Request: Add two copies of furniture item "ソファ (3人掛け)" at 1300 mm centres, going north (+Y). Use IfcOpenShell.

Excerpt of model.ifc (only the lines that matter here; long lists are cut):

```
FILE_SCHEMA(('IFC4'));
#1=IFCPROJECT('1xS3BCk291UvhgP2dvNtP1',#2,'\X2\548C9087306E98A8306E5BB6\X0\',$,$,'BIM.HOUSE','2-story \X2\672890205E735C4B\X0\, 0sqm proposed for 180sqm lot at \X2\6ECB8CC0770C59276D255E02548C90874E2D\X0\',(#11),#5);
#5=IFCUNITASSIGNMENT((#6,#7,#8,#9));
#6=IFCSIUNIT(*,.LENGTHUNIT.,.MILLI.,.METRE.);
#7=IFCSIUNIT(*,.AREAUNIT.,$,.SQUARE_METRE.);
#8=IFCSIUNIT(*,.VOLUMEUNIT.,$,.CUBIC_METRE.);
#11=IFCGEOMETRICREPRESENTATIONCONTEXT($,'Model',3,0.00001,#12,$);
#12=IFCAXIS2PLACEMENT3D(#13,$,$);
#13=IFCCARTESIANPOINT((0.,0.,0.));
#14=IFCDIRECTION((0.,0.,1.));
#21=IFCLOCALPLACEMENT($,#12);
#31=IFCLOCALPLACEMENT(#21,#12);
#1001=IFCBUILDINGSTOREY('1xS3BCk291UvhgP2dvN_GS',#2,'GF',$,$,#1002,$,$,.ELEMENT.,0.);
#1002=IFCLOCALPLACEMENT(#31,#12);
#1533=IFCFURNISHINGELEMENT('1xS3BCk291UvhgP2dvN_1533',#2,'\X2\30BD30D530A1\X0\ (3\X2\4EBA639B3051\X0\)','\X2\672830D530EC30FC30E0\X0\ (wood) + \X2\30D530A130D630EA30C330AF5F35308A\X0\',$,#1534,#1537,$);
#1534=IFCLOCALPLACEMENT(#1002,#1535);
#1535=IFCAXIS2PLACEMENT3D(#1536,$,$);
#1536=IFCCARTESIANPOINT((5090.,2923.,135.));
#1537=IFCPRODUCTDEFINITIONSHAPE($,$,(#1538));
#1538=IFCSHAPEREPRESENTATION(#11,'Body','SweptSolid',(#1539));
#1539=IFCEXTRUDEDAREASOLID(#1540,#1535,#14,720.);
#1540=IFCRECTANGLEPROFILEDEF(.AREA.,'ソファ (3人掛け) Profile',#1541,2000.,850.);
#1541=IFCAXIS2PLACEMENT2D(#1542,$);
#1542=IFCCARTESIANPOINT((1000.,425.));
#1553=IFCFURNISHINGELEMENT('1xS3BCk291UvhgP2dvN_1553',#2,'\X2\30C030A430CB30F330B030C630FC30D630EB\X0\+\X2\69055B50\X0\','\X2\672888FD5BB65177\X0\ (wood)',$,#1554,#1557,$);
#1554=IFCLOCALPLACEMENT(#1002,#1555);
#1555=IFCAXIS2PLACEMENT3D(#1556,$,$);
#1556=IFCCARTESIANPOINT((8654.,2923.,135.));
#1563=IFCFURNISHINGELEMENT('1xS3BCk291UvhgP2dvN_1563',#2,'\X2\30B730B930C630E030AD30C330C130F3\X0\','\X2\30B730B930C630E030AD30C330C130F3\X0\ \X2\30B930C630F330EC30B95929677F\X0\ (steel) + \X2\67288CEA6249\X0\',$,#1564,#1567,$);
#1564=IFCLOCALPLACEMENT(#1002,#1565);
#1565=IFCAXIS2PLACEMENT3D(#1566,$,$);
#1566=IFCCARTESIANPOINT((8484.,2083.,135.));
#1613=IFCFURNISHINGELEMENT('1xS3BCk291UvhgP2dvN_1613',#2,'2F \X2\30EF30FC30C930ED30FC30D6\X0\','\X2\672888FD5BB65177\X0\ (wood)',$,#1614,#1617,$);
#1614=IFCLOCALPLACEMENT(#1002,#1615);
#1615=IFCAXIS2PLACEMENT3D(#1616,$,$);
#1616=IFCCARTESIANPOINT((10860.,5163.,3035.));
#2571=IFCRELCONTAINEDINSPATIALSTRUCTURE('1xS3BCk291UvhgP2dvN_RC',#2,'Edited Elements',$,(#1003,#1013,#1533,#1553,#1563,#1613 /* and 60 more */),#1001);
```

```python
import numpy as np
import ifcopenshell
import ifcopenshell.api.geometry
import ifcopenshell.api.root
import ifcopenshell.util.element
import ifcopenshell.util.placement

model = ifcopenshell.open("model.ifc")


def reuse_history(source, copy):
    """copy_class also copies each property set's owner history, people and application; keep the originals."""
    for rel in copy.IsDefinedBy:
        if rel.is_a("IfcRelDefinesByProperties") and (history := rel.RelatingPropertyDefinition.OwnerHistory):
            rel.RelatingPropertyDefinition.OwnerHistory = source.OwnerHistory
            ifcopenshell.util.element.remove_deep2(model, history)


source = model.by_guid("1xS3BCk291UvhgP2dvN_1533")
base = ifcopenshell.util.placement.get_local_placement(source.ObjectPlacement)
step = np.array([0.0, 1.0, 0.0]) * 1300.0

for i in range(1, 3):
    copy = ifcopenshell.api.root.copy_class(model, product=source)
    copy.Representation = ifcopenshell.util.element.copy_deep(
        model, source.Representation, exclude=["IfcGeometricRepresentationContext", "IfcRepresentationMap"]
    )
    reuse_history(source, copy)
    matrix = base.copy()
    matrix[:3, 3] += i * step
    print("added at", matrix[:3, 3].round(3) + 0.0)
    ifcopenshell.api.geometry.edit_object_placement(model, product=copy, matrix=matrix, is_si=False)

model.write("model-out.ifc")
```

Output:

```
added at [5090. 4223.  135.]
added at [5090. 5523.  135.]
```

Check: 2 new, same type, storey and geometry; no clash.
